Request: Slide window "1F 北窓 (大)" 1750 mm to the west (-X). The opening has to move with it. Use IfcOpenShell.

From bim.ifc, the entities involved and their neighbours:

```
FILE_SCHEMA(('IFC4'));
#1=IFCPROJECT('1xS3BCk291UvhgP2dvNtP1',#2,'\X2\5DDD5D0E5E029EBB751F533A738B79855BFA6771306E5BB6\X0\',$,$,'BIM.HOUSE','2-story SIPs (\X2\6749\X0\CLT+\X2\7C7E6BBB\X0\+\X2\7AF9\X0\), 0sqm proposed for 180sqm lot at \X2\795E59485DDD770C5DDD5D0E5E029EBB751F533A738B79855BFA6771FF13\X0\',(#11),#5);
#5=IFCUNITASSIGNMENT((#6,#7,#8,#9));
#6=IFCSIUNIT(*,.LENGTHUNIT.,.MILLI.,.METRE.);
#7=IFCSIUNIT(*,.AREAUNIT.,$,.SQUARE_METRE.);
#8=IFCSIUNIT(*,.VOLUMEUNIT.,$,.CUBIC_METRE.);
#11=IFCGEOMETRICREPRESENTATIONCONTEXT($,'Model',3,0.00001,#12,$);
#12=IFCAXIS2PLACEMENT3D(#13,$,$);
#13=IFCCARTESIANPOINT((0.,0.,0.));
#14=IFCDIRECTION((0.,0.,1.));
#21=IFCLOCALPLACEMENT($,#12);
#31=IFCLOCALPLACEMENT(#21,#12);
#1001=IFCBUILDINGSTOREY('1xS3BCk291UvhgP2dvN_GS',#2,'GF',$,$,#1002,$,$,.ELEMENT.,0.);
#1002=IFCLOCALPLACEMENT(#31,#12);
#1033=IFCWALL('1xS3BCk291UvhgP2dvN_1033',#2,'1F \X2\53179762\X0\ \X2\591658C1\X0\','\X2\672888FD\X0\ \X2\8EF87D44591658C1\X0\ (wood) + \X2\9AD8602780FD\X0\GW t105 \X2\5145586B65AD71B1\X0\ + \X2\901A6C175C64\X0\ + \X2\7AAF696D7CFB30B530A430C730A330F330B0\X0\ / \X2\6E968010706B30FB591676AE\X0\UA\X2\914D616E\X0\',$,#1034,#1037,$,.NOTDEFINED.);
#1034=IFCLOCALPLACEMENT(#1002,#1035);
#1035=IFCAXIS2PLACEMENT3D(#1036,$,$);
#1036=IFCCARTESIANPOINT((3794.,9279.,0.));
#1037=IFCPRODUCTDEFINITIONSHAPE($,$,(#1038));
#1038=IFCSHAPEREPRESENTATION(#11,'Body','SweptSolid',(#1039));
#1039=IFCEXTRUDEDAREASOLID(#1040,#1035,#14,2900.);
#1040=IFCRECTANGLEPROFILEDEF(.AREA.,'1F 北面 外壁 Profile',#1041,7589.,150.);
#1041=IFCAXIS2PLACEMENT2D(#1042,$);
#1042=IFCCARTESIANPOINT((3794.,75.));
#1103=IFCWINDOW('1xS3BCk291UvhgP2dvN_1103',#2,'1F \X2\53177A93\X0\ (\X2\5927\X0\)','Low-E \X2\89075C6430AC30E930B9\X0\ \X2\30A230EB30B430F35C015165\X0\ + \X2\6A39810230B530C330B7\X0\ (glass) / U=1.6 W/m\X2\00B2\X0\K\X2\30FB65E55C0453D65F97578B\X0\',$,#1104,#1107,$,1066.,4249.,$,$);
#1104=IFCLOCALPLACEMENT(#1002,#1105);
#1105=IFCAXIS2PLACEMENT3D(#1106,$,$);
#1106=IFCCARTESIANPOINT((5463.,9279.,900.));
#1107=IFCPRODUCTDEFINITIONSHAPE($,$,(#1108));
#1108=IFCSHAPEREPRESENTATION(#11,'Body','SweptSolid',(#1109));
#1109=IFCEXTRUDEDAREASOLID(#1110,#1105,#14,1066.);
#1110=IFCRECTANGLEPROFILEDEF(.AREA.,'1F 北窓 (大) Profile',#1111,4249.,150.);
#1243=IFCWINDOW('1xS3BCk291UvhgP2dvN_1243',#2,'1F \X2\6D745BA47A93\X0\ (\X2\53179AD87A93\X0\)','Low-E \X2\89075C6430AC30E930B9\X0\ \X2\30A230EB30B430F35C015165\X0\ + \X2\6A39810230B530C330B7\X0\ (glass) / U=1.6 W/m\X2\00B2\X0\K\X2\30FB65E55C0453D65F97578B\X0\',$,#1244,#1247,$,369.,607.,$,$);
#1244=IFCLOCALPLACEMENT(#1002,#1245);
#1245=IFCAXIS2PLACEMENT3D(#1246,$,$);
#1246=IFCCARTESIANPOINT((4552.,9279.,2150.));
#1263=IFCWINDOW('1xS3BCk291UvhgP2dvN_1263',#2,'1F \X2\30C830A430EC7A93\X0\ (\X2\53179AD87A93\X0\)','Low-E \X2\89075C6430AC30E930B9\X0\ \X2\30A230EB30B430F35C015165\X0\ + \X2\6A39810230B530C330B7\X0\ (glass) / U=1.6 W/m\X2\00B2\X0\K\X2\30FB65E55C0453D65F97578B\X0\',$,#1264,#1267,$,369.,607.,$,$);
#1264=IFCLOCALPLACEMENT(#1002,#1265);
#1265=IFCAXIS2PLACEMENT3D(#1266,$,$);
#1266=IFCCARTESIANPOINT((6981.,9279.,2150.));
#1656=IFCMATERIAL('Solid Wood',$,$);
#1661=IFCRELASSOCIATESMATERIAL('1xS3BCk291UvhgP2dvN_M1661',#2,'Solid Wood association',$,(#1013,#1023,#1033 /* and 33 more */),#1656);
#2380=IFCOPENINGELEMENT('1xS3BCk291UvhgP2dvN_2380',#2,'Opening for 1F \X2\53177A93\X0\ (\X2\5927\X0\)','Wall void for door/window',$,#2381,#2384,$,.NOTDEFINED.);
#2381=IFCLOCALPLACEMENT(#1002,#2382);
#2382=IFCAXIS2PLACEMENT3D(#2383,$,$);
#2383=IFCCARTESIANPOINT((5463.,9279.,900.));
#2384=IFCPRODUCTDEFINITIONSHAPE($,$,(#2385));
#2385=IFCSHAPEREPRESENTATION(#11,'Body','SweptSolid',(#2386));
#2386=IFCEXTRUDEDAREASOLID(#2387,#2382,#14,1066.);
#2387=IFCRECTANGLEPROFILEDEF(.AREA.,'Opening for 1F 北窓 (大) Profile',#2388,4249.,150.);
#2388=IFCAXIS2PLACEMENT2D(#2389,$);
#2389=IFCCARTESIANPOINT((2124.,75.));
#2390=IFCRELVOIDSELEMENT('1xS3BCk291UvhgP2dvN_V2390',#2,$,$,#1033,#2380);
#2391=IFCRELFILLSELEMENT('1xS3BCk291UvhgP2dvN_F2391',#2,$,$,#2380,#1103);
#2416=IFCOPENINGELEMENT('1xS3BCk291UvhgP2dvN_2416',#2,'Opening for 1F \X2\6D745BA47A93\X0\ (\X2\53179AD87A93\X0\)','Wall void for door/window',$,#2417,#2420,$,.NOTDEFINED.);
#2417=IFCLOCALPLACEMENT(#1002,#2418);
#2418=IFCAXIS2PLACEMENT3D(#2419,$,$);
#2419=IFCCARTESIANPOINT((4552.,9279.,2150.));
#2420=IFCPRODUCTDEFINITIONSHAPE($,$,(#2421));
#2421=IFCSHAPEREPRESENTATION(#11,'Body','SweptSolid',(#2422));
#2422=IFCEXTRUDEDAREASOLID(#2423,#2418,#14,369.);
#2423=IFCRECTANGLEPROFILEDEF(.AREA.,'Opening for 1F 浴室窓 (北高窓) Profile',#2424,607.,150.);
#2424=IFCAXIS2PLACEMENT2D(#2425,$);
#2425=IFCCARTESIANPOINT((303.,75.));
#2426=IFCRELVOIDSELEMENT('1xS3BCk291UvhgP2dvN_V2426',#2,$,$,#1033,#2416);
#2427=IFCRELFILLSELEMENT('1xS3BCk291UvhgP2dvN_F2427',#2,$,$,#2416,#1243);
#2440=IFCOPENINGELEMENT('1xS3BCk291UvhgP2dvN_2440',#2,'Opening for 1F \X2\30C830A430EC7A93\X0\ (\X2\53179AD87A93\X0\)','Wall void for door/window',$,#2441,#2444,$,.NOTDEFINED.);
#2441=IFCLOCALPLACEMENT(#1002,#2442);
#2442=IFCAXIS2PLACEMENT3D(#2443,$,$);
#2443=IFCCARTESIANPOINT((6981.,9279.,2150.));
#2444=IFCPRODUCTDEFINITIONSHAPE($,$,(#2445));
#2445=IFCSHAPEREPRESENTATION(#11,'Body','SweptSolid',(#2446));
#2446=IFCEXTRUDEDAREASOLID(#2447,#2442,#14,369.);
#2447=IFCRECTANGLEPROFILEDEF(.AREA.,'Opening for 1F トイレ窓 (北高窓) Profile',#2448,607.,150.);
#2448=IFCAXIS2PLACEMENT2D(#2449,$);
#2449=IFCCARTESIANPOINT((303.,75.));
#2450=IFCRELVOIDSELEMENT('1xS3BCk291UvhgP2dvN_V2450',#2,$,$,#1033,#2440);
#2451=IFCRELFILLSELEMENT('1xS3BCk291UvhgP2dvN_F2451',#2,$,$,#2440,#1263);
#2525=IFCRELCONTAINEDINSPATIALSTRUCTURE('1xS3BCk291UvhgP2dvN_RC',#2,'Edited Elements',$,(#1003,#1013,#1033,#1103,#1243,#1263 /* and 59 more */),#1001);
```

```python
import ifcopenshell
import ifcopenshell.api.geometry
import ifcopenshell.util.placement

model = ifcopenshell.open("bim.ifc")

window = model.by_guid("1xS3BCk291UvhgP2dvN_1103")
opening = window.FillsVoids[0].RelatingOpeningElement
wall = opening.VoidsElements[0].RelatingBuildingElement

wall_matrix = ifcopenshell.util.placement.get_local_placement(wall.ObjectPlacement)
shift = wall_matrix[:3, 0] * -1750.0
before = ifcopenshell.util.placement.get_local_placement(window.ObjectPlacement)[:3, 3].copy()

# The window is not placed relative to its opening, so move both.
for product in (opening, window):
    matrix = ifcopenshell.util.placement.get_local_placement(product.ObjectPlacement)
    matrix[:3, 3] += shift
    ifcopenshell.api.geometry.edit_object_placement(model, product=product, matrix=matrix, is_si=False)

after = ifcopenshell.util.placement.get_local_placement(window.ObjectPlacement)[:3, 3]
print("window moved by", (after - before).round(3) + 0.0)

model.write("bim_rev.ifc")
```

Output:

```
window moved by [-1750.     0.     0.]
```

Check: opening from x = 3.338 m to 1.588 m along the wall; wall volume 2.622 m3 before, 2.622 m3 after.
